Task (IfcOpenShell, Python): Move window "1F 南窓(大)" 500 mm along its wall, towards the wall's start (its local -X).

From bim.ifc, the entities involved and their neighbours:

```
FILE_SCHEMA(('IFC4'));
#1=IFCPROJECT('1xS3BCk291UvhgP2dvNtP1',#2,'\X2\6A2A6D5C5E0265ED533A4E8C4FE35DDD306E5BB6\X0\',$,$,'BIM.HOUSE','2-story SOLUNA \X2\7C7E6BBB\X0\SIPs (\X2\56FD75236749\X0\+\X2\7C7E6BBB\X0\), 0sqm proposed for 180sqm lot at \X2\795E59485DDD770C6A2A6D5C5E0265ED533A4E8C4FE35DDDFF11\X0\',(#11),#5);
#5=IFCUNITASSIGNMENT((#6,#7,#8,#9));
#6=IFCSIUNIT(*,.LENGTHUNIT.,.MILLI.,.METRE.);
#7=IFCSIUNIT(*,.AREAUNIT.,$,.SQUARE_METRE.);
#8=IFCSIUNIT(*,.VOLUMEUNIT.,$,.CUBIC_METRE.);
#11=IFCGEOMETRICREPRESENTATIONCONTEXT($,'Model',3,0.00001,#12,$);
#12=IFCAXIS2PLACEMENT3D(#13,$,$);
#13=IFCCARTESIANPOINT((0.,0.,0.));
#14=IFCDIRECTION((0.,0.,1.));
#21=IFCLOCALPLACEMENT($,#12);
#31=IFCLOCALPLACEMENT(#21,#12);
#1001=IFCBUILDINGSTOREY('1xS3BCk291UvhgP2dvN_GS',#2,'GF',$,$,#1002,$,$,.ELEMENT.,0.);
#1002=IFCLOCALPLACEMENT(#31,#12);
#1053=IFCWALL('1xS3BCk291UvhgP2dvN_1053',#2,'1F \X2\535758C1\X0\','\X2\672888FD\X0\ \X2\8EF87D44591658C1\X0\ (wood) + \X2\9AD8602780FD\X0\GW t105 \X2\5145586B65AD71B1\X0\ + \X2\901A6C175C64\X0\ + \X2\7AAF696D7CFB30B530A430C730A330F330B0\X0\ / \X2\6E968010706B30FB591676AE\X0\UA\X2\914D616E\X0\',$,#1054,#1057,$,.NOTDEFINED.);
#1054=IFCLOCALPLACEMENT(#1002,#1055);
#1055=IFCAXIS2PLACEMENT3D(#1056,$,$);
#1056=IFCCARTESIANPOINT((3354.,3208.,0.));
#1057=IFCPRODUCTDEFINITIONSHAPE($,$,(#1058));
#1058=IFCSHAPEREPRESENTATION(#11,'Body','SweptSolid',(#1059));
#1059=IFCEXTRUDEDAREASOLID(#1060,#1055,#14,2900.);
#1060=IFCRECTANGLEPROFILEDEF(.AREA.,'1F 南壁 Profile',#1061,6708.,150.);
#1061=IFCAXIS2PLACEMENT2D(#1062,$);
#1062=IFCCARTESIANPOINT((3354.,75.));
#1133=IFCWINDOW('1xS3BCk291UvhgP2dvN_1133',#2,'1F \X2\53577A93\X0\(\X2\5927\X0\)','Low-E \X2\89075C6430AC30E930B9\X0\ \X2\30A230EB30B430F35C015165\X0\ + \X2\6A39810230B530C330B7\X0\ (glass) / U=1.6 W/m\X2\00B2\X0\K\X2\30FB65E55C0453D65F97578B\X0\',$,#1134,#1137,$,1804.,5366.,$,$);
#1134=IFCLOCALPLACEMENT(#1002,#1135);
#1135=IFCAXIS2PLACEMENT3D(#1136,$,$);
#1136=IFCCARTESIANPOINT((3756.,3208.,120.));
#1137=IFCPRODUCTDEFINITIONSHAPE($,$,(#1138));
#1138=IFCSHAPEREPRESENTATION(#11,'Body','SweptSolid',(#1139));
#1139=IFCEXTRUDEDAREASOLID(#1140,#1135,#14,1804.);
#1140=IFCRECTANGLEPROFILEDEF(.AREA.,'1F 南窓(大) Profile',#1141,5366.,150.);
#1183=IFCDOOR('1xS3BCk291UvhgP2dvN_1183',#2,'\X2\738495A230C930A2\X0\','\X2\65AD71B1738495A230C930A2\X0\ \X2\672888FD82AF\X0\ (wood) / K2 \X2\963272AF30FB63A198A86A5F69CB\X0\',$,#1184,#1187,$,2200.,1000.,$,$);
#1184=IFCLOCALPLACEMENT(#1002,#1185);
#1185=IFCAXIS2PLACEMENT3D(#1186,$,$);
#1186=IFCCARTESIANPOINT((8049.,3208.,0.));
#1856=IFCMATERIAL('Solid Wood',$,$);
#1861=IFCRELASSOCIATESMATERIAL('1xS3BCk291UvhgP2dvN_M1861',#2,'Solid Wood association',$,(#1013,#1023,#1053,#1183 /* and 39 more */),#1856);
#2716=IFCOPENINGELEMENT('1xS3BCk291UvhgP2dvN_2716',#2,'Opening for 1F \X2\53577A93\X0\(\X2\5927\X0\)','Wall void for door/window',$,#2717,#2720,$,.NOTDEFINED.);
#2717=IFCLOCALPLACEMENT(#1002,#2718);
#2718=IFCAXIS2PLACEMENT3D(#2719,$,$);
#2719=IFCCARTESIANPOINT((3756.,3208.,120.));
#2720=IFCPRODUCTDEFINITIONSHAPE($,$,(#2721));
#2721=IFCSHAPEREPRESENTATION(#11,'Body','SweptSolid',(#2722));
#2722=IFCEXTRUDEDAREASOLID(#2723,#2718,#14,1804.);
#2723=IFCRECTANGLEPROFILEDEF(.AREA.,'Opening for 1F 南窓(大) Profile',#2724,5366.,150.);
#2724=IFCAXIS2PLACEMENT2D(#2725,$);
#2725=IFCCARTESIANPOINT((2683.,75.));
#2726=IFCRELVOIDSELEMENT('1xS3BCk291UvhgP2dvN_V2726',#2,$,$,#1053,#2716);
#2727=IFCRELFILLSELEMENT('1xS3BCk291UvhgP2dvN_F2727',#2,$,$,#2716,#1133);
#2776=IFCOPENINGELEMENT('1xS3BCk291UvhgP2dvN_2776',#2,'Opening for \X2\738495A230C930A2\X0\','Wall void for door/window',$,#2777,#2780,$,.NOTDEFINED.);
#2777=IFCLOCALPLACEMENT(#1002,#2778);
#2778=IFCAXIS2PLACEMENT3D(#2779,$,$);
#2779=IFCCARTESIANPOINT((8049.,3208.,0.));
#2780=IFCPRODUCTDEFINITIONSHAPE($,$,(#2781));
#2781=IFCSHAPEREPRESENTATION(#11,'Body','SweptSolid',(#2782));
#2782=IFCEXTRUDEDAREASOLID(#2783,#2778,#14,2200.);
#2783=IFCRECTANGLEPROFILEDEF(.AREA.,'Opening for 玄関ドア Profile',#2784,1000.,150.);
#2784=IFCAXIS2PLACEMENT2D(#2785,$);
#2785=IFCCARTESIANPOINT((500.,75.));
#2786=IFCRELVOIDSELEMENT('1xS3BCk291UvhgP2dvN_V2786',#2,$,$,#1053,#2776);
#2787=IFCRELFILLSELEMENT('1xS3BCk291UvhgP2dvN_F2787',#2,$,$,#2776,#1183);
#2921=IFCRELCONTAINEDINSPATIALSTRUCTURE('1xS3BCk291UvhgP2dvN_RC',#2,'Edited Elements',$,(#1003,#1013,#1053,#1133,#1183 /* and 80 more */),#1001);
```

```python
import ifcopenshell
import ifcopenshell.api.geometry
import ifcopenshell.util.placement

model = ifcopenshell.open("bim.ifc")

window = model.by_id(1133)
opening = window.FillsVoids[0].RelatingOpeningElement
wall = opening.VoidsElements[0].RelatingBuildingElement

wall_matrix = ifcopenshell.util.placement.get_local_placement(wall.ObjectPlacement)
shift = wall_matrix[:3, 0] * -500.0
before = ifcopenshell.util.placement.get_local_placement(window.ObjectPlacement)[:3, 3].copy()

# The window is not placed relative to its opening, so move both.
for product in (opening, window):
    matrix = ifcopenshell.util.placement.get_local_placement(product.ObjectPlacement)
    matrix[:3, 3] += shift
    ifcopenshell.api.geometry.edit_object_placement(model, product=product, matrix=matrix, is_si=False)

after = ifcopenshell.util.placement.get_local_placement(window.ObjectPlacement)[:3, 3]
print("window moved by", (after - before).round(3) + 0.0)

model.write("bim_edited.ifc")
```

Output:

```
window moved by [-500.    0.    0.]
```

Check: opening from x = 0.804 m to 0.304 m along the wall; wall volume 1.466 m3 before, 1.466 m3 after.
